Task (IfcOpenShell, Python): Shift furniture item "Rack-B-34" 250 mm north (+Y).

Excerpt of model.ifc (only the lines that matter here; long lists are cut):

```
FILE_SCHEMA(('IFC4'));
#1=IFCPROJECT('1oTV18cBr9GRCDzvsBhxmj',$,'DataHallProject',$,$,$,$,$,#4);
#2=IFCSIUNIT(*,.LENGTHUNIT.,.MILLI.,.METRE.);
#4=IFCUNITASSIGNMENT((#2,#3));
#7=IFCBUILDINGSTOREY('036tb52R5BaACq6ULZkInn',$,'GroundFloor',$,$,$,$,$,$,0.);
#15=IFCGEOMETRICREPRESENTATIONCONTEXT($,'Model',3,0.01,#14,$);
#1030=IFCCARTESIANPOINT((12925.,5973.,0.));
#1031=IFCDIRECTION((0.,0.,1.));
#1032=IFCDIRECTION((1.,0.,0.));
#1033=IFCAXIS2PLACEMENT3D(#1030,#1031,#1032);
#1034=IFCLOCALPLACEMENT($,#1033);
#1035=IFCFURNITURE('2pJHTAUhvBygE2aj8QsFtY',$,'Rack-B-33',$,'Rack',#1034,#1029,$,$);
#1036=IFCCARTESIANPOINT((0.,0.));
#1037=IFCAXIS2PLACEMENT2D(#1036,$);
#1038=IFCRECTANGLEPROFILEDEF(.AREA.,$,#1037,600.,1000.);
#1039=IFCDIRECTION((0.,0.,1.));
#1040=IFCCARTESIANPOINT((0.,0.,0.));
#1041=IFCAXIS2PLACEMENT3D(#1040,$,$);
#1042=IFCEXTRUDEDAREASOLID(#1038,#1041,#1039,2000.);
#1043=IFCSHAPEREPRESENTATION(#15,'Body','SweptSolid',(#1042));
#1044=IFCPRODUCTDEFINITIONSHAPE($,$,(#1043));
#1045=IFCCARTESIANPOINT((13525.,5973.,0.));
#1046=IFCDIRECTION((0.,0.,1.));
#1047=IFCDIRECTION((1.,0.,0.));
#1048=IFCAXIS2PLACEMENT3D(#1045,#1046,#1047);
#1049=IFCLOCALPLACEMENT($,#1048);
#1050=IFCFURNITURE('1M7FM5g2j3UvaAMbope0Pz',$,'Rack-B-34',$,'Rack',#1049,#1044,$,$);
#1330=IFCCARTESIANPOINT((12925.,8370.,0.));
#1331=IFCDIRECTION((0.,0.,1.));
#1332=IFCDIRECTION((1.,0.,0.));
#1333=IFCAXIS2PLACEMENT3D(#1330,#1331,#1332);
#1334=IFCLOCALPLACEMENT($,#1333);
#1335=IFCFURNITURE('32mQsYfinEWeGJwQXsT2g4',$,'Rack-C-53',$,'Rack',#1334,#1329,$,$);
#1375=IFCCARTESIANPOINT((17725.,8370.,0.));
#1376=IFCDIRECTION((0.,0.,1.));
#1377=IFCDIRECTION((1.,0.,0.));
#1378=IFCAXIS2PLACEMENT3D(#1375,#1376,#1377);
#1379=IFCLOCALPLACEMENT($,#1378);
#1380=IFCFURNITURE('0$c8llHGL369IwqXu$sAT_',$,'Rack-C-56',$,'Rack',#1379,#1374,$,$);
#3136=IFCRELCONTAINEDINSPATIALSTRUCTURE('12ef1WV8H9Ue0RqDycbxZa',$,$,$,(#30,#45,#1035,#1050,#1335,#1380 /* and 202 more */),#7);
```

```python
import ifcopenshell
import ifcopenshell.api.geometry
import ifcopenshell.util.placement

model = ifcopenshell.open("model.ifc")

item = model.by_guid("1M7FM5g2j3UvaAMbope0Pz")
matrix = ifcopenshell.util.placement.get_local_placement(item.ObjectPlacement)
matrix[1, 3] += 250.0
ifcopenshell.api.geometry.edit_object_placement(model, product=item, matrix=matrix, is_si=False)

print(ifcopenshell.util.placement.get_local_placement(item.ObjectPlacement).round(3) + 0.0)

model.write("model-out.ifc")
```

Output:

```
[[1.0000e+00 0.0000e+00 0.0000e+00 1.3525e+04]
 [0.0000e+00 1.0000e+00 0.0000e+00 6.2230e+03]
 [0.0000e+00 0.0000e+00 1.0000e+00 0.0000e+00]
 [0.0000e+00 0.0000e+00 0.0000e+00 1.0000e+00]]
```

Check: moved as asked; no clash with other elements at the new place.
